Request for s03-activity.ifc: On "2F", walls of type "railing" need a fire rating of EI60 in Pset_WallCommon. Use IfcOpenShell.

First a look at what the model holds.

```python
import ifcopenshell
import ifcopenshell.util.element

model = ifcopenshell.open("s03-activity.ifc")
print(model.schema)
storey = next(s for s in model.by_type("IfcBuildingStorey") if s.Name == "2F")
walls = [e for e in ifcopenshell.util.element.get_decomposition(storey) if e.is_a("IfcWall")]
seen = {}
for e in walls:
    element_type = ifcopenshell.util.element.get_type(e)
    key = (element_type.Name if element_type != e and element_type else None, ifcopenshell.util.element.get_pset(e, "Pset_WallCommon", "FireRating"))
    seen[key] = seen.get(key, 0) + 1
for (name, value), count in sorted(seen.items(), key=str):
    print(count, "x", name, "|", value)
```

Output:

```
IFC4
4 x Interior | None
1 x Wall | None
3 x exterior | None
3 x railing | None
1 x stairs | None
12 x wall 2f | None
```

```python
import ifcopenshell
import ifcopenshell.api.pset
import ifcopenshell.util.element

model = ifcopenshell.open("s03-activity.ifc")

storey = next(s for s in model.by_type("IfcBuildingStorey") if s.Name == "2F")
walls = [e for e in ifcopenshell.util.element.get_decomposition(storey) if e.is_a("IfcWall")]

count = 0
for e in walls:
    element_type = ifcopenshell.util.element.get_type(e)
    if element_type in (None, e) or element_type.Name != "railing":
        continue
    # add_pset returns the element's existing set when there is one.
    pset = ifcopenshell.api.pset.add_pset(model, product=e, name="Pset_WallCommon")
    ifcopenshell.api.pset.edit_pset(model, pset=pset, properties={"FireRating": "EI60"})
    count += 1

print(count, "walls updated")

model.write("s03-activity_edited.ifc")
```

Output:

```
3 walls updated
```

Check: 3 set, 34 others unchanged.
